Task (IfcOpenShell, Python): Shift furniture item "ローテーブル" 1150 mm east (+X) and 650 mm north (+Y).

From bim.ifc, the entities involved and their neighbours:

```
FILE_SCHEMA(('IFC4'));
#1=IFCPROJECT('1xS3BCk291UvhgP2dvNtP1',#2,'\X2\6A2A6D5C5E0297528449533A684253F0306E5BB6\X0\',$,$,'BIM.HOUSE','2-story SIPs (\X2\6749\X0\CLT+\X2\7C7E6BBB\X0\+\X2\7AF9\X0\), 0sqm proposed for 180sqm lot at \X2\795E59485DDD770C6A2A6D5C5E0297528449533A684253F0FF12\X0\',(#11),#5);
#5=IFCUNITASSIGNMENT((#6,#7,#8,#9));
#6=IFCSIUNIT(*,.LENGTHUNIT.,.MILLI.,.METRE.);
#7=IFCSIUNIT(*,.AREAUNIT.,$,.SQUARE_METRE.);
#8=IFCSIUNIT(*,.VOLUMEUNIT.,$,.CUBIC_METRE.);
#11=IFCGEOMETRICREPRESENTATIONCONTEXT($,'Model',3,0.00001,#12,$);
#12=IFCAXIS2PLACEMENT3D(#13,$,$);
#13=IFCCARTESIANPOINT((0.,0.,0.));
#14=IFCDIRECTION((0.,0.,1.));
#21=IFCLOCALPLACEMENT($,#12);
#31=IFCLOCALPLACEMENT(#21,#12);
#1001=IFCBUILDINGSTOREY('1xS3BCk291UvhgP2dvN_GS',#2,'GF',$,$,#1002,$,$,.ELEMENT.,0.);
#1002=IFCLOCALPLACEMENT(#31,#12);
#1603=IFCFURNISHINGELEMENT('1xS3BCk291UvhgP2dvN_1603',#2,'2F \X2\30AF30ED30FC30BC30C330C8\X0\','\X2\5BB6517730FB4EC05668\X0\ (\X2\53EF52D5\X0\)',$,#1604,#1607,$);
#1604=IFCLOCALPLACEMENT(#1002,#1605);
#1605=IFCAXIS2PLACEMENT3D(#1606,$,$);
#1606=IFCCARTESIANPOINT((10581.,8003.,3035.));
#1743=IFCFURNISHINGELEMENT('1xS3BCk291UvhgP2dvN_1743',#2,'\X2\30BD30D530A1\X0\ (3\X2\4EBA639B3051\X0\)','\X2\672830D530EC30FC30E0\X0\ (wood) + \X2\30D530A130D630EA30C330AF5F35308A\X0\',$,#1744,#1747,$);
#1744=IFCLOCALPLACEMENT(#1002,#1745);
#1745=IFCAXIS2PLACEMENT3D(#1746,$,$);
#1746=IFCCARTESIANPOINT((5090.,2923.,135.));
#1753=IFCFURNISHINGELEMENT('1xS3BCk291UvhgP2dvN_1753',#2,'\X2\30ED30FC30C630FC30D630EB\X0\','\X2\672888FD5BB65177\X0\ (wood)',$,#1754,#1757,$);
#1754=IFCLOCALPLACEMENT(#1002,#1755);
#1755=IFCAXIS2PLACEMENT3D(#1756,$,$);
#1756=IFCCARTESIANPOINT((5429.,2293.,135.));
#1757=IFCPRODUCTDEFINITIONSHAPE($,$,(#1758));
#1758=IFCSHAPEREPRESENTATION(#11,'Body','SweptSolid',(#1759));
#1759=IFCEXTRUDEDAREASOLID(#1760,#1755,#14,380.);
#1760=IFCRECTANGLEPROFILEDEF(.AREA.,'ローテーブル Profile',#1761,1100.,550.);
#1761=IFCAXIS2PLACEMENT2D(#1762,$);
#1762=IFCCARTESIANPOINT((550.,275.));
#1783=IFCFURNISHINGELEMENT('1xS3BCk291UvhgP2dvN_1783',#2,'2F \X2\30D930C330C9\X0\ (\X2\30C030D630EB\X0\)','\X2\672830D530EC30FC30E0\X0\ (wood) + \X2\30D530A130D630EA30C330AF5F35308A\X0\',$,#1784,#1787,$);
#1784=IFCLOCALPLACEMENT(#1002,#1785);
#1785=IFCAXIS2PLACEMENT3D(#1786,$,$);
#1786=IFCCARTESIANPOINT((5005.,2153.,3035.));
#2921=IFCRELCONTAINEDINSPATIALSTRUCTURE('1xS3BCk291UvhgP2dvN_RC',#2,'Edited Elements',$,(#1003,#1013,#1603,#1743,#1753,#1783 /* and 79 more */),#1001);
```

```python
import ifcopenshell
import ifcopenshell.api.geometry
import ifcopenshell.util.placement

model = ifcopenshell.open("bim.ifc")

item = model.by_guid("1xS3BCk291UvhgP2dvN_1753")
matrix = ifcopenshell.util.placement.get_local_placement(item.ObjectPlacement)
matrix[0, 3] += 1150.0
matrix[1, 3] += 650.0
ifcopenshell.api.geometry.edit_object_placement(model, product=item, matrix=matrix, is_si=False)

print(ifcopenshell.util.placement.get_local_placement(item.ObjectPlacement).round(3) + 0.0)

model.write("bim_rev.ifc")
```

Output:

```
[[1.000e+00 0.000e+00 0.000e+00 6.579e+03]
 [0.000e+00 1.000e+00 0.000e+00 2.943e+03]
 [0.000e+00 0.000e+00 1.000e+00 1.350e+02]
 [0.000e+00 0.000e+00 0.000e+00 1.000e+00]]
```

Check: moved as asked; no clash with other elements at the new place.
